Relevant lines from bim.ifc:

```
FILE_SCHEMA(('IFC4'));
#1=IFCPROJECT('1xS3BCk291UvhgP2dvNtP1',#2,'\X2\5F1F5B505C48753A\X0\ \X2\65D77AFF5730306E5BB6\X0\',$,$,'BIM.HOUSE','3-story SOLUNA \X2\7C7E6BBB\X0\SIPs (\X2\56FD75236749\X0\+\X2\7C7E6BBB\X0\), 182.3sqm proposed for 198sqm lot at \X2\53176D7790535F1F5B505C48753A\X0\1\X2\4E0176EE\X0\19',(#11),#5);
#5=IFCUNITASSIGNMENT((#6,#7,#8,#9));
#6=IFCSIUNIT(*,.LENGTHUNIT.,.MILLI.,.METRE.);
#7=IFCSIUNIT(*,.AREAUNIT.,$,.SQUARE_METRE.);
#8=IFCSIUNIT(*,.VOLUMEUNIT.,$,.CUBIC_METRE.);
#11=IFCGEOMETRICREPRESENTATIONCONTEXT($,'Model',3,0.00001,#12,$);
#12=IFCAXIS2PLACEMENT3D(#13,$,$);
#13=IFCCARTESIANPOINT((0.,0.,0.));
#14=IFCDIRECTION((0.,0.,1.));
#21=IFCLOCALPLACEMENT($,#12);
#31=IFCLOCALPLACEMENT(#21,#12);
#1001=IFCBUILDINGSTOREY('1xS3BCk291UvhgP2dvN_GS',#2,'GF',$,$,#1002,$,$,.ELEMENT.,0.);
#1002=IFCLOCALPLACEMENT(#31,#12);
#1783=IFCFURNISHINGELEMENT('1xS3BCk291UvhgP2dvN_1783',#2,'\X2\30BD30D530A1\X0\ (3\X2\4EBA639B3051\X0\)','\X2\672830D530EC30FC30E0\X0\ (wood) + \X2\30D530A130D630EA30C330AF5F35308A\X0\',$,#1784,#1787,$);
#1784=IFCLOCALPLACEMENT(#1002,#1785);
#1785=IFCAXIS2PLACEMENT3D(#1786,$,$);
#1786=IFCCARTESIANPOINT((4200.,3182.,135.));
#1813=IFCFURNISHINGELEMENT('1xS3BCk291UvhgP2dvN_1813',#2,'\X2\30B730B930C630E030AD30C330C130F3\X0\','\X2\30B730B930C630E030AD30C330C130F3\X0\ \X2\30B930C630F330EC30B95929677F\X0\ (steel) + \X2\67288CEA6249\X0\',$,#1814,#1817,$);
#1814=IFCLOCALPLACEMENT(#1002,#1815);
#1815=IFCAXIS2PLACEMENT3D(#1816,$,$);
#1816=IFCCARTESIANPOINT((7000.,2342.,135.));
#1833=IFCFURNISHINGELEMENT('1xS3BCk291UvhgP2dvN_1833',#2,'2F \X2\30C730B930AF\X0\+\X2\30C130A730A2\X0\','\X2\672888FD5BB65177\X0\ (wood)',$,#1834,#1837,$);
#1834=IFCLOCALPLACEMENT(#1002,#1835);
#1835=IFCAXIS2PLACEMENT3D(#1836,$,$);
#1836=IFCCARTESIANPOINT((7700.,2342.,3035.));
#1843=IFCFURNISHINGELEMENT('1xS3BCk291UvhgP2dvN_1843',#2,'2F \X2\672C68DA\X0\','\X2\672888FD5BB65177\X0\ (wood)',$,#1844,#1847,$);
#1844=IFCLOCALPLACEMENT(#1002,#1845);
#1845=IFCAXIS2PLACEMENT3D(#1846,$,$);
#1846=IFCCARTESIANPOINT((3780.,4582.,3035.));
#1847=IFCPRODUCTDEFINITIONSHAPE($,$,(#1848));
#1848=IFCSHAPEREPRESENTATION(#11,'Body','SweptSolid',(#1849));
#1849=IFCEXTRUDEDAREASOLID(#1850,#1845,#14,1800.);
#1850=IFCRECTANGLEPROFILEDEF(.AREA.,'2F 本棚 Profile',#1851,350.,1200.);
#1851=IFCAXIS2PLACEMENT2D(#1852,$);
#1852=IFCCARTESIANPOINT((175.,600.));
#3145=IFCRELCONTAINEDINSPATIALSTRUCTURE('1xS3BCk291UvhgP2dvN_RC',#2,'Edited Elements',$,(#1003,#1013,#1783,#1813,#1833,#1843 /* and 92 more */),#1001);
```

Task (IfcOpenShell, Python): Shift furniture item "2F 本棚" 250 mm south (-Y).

```python
import ifcopenshell
import ifcopenshell.api.geometry
import ifcopenshell.util.placement
import ifcopenshell.util.unit

model = ifcopenshell.open("bim.ifc")
unit_scale = ifcopenshell.util.unit.calculate_unit_scale(model)

item = model.by_id(1843)
matrix = ifcopenshell.util.placement.get_local_placement(item.ObjectPlacement)
matrix[1, 3] -= 0.25 / unit_scale
ifcopenshell.api.geometry.edit_object_placement(model, product=item, matrix=matrix, is_si=False)

print(ifcopenshell.util.placement.get_local_placement(item.ObjectPlacement).round(3) + 0.0)

model.write("bim-out.ifc")
```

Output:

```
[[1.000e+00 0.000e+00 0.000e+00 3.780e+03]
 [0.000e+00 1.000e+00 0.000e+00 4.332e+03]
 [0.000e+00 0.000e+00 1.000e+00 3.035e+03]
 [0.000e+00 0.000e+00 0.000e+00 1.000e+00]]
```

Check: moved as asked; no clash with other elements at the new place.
